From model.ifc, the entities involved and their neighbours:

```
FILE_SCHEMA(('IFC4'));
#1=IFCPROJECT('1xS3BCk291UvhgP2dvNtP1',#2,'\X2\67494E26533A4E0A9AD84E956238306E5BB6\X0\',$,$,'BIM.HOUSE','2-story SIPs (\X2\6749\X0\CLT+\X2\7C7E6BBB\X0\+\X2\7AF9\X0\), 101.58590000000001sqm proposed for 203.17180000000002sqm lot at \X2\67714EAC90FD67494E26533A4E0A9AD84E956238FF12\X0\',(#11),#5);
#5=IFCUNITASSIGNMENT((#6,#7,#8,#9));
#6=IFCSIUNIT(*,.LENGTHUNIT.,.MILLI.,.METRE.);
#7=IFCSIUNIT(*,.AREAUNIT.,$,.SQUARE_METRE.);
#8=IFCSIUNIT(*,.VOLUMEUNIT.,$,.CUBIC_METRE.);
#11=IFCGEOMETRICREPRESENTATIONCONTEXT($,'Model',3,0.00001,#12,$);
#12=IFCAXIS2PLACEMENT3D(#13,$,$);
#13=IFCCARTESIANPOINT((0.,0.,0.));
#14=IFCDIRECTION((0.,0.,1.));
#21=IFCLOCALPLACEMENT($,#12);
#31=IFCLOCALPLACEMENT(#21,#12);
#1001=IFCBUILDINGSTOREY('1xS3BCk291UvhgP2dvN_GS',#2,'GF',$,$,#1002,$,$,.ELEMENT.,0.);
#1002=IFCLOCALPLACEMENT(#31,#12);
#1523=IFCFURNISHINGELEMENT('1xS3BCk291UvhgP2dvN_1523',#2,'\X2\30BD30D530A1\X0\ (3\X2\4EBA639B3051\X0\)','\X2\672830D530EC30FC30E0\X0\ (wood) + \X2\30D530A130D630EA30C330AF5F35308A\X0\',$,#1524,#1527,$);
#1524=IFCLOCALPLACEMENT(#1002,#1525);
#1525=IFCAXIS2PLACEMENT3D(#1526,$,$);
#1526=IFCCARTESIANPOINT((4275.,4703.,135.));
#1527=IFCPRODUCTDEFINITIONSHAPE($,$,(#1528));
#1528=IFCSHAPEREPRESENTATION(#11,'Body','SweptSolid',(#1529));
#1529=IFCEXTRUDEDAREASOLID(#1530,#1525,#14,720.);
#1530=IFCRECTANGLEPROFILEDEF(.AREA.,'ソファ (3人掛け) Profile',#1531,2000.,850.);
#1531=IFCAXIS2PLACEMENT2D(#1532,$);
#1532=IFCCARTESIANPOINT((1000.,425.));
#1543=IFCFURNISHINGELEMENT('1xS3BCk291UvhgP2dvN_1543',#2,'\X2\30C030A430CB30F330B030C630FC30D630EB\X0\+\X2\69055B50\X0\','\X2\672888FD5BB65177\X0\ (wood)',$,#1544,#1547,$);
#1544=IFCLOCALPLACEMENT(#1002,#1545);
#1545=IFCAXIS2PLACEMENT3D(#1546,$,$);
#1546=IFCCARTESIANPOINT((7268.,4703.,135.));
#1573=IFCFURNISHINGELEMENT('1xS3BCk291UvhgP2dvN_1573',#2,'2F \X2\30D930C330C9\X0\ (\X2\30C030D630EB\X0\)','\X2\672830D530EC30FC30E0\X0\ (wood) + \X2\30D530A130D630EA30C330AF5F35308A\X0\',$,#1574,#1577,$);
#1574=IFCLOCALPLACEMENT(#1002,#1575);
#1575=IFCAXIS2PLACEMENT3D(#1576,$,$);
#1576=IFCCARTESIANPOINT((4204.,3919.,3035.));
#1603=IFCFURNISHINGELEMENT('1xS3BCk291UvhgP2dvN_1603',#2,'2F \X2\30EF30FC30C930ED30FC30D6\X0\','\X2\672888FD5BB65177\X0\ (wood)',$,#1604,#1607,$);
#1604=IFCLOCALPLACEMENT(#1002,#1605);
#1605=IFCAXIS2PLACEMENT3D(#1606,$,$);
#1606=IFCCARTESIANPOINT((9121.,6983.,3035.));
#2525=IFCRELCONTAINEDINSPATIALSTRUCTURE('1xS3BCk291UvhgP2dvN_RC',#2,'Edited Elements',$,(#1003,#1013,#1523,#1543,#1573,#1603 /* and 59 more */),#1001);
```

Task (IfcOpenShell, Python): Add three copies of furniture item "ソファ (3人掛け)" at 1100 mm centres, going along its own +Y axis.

```python
import ifcopenshell
import ifcopenshell.api.geometry
import ifcopenshell.api.root
import ifcopenshell.util.element
import ifcopenshell.util.placement
import ifcopenshell.util.unit

model = ifcopenshell.open("model.ifc")
unit_scale = ifcopenshell.util.unit.calculate_unit_scale(model)


def reuse_history(source, copy):
    """copy_class also copies each property set's owner history, people and application; keep the originals."""
    for rel in copy.IsDefinedBy:
        if rel.is_a("IfcRelDefinesByProperties") and (history := rel.RelatingPropertyDefinition.OwnerHistory):
            rel.RelatingPropertyDefinition.OwnerHistory = source.OwnerHistory
            ifcopenshell.util.element.remove_deep2(model, history)


source = model.by_id(1523)
base = ifcopenshell.util.placement.get_local_placement(source.ObjectPlacement)
step = base[:3, 1] * 1.1 / unit_scale

for i in range(1, 4):
    copy = ifcopenshell.api.root.copy_class(model, product=source)
    copy.Representation = ifcopenshell.util.element.copy_deep(
        model, source.Representation, exclude=["IfcGeometricRepresentationContext", "IfcRepresentationMap"]
    )
    reuse_history(source, copy)
    matrix = base.copy()
    matrix[:3, 3] += i * step
    print("added at", matrix[:3, 3].round(3) + 0.0)
    ifcopenshell.api.geometry.edit_object_placement(model, product=copy, matrix=matrix, is_si=False)

model.write("model_updated.ifc")
```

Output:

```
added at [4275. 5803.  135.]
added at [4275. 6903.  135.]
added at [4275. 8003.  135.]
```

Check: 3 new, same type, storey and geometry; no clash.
